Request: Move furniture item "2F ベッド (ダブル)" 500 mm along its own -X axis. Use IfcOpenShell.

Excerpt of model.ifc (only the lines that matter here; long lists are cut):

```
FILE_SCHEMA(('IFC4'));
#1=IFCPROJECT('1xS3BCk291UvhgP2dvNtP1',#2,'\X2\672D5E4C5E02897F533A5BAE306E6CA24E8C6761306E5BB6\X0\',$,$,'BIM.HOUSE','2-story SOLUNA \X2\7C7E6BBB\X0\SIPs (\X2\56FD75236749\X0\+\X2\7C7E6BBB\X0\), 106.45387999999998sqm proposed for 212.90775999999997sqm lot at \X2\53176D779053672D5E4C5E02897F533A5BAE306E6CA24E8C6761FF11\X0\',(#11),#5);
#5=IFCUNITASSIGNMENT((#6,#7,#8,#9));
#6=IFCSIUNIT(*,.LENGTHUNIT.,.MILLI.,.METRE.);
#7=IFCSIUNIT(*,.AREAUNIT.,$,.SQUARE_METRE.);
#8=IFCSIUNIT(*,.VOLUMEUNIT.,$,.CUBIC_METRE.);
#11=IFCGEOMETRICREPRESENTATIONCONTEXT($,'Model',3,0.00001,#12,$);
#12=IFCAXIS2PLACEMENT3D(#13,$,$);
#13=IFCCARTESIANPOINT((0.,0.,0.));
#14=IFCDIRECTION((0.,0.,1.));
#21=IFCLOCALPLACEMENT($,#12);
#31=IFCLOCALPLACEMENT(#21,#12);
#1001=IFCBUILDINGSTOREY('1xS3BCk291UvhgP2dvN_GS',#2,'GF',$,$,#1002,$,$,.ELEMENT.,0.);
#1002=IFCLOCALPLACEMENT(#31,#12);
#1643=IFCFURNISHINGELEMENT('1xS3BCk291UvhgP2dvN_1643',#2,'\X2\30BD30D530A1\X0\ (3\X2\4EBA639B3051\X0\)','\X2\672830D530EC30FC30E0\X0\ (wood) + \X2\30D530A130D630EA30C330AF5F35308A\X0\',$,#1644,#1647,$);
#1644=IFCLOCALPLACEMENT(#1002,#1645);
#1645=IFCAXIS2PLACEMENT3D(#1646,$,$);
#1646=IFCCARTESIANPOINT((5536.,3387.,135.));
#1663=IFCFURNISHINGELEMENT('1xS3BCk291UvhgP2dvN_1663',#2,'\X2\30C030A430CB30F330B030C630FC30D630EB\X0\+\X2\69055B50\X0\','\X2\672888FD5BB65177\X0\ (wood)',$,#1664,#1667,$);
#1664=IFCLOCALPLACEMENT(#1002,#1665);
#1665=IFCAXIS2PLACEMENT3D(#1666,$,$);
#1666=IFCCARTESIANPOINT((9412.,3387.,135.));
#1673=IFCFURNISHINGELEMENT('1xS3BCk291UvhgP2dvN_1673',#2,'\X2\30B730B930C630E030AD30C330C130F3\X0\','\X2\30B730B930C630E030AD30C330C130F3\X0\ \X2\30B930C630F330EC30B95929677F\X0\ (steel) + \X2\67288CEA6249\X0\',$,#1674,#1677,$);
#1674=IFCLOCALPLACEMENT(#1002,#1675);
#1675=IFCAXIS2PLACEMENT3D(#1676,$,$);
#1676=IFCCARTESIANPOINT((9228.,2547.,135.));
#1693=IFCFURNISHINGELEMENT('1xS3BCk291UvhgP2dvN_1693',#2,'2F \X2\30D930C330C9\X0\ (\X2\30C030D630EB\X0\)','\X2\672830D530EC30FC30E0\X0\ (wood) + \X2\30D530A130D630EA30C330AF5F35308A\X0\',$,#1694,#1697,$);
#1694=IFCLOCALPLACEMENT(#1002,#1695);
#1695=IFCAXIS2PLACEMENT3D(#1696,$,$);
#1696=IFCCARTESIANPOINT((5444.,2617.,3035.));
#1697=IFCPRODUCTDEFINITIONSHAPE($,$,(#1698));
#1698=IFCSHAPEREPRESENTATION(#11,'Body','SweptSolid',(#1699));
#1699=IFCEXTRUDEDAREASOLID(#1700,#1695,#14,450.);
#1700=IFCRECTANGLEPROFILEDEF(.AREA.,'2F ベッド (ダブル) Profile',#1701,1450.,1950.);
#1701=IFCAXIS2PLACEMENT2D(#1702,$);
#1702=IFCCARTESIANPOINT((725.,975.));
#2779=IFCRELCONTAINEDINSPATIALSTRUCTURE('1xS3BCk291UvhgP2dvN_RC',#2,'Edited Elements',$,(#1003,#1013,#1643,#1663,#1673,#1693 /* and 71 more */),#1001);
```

```python
import ifcopenshell
import ifcopenshell.api.geometry
import ifcopenshell.util.placement
import ifcopenshell.util.unit

model = ifcopenshell.open("model.ifc")
unit_scale = ifcopenshell.util.unit.calculate_unit_scale(model)

item = model.by_guid("1xS3BCk291UvhgP2dvN_1693")
matrix = ifcopenshell.util.placement.get_local_placement(item.ObjectPlacement)
matrix[:3, 3] -= matrix[:3, 0] * 0.5 / unit_scale
ifcopenshell.api.geometry.edit_object_placement(model, product=item, matrix=matrix, is_si=False)

print(ifcopenshell.util.placement.get_local_placement(item.ObjectPlacement).round(3) + 0.0)

model.write("model_v2.ifc")
```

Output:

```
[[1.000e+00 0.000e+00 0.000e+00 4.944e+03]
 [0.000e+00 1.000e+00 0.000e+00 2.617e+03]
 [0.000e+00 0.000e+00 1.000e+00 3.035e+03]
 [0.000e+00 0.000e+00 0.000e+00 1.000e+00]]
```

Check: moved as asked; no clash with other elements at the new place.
